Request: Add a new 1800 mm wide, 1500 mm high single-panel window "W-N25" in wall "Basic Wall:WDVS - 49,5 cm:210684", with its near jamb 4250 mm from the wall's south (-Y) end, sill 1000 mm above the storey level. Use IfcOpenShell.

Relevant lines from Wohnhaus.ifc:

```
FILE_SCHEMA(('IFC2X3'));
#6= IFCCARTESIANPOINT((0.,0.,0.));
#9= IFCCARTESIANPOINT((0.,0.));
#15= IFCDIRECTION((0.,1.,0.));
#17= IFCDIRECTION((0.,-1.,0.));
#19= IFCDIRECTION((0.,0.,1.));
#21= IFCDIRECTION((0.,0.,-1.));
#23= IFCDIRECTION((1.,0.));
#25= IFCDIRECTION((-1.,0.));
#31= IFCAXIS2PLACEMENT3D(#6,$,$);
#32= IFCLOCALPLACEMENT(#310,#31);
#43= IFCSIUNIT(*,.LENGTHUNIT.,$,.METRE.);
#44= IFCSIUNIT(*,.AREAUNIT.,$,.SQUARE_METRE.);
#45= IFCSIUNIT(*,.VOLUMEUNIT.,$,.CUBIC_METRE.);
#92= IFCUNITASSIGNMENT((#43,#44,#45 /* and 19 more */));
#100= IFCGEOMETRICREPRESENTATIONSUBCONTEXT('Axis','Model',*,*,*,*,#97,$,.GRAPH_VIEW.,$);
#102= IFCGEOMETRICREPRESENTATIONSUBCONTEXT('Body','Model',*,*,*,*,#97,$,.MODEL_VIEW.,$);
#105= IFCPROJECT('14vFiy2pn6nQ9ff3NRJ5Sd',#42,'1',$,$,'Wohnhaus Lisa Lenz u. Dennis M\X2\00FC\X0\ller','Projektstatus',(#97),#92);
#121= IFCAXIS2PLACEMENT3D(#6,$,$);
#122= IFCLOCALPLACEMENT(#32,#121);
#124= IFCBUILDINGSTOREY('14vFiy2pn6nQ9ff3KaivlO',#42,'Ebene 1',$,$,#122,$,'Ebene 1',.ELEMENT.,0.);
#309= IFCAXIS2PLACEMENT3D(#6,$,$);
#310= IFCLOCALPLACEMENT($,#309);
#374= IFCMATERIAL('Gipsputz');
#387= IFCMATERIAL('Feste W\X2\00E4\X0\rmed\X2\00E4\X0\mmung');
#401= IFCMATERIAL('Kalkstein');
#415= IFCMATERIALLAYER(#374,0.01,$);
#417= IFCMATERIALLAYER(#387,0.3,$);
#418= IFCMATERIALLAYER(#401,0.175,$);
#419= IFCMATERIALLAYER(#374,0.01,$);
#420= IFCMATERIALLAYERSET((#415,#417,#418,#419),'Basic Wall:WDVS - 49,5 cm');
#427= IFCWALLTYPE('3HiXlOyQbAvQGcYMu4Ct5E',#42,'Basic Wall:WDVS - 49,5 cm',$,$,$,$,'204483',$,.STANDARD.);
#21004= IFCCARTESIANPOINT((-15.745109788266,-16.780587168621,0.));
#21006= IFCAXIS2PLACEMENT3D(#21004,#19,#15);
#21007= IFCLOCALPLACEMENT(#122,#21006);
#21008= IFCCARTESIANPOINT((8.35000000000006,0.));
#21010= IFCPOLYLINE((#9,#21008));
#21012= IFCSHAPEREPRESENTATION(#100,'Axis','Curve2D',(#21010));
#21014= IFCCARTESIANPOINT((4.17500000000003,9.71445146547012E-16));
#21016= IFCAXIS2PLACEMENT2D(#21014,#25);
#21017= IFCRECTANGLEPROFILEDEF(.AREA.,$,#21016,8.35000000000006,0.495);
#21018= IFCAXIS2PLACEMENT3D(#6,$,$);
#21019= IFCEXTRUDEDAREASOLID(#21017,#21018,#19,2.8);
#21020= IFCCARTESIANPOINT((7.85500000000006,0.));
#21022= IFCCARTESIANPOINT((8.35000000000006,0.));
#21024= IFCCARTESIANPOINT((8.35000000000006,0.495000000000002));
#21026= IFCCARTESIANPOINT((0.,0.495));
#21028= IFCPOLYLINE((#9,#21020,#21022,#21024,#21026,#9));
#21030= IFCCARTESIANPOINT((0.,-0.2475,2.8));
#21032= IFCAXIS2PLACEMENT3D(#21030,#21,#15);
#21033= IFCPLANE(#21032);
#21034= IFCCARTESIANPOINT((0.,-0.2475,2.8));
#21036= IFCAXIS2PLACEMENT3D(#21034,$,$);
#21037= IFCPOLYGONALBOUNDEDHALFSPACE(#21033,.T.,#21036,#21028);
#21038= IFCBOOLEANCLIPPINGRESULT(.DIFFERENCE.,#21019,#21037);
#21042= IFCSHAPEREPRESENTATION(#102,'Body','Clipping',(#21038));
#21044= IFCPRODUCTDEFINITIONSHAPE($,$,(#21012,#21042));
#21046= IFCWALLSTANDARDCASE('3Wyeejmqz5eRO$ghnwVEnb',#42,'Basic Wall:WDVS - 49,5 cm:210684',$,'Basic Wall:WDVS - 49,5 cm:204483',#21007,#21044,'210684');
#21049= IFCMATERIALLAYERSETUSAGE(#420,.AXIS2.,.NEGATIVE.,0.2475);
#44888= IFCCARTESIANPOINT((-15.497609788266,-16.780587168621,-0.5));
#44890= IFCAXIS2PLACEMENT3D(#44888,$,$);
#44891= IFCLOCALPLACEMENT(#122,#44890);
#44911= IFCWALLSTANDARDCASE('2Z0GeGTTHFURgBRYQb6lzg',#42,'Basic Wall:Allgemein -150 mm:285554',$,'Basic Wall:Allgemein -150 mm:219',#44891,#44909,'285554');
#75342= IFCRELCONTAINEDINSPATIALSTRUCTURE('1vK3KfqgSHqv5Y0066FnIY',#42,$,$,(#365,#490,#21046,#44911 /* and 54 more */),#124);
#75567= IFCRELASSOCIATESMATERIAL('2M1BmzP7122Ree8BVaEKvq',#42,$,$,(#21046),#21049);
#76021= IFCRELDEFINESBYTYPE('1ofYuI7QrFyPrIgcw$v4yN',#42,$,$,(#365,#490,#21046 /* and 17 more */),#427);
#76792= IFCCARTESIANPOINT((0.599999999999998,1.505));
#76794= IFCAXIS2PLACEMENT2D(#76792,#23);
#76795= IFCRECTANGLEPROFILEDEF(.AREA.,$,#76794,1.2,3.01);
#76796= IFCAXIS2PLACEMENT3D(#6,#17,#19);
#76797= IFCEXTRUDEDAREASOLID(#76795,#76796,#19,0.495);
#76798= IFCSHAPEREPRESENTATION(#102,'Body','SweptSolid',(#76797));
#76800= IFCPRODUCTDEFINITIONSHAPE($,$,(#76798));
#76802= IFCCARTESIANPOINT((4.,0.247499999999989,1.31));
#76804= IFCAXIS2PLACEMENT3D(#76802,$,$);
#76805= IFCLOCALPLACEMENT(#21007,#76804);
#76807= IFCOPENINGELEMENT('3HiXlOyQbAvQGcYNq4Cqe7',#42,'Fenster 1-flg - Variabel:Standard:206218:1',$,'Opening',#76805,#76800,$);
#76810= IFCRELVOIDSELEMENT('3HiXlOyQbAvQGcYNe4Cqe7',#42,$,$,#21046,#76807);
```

```python
import numpy as np
import ifcopenshell
import ifcopenshell.api.feature
import ifcopenshell.api.geometry
import ifcopenshell.api.root
import ifcopenshell.api.spatial
import ifcopenshell.api.type
import ifcopenshell.geom
import ifcopenshell.util.element
import ifcopenshell.util.placement
import ifcopenshell.util.representation
import ifcopenshell.util.shape
import ifcopenshell.util.unit

model = ifcopenshell.open("Wohnhaus.ifc")
unit_scale = ifcopenshell.util.unit.calculate_unit_scale(model)
settings = ifcopenshell.geom.settings()


def volume(element):
    """Net volume in cubic metres, openings subtracted."""
    shape = ifcopenshell.geom.create_shape(settings, element)
    return ifcopenshell.util.shape.get_volume(shape.geometry)


wall = model.by_guid("3Wyeejmqz5eRO$ghnwVEnb")
storey = ifcopenshell.util.element.get_container(wall, ifc_class="IfcBuildingStorey")
context = ifcopenshell.util.representation.get_context(model, "Model", "Body", "MODEL_VIEW")
before = volume(wall)

width, height, from_end, sill = 1.8, 1.5, 4.25, 1  # metres

# The wall runs along its own X axis, and the end named is its -X end.
wall_shape = ifcopenshell.geom.create_shape(settings, wall)
x, y, z = ifcopenshell.util.shape.get_vertices(wall_shape.geometry).T
start = x.min() + from_end
face, thickness = float(y.min()), float(y.max() - y.min())
wall_matrix = ifcopenshell.util.placement.get_local_placement(wall.ObjectPlacement)
level = ifcopenshell.util.placement.get_local_placement(storey.ObjectPlacement)[2, 3]


def in_wall(x, y):
    """Placement at x, y metres in the wall's axes, at sill height."""
    matrix = wall_matrix.copy()
    matrix[:, 3] = wall_matrix @ np.array([x / unit_scale, y / unit_scale, 0.0, 1.0])
    matrix[2, 3] = level + sill / unit_scale
    return matrix


# Opening: a box that overshoots both wall faces by 50 mm.
opening = ifcopenshell.api.root.create_entity(model, ifc_class="IfcOpeningElement")
box = ifcopenshell.api.geometry.add_wall_representation(
    model, context=context, length=width, height=height, thickness=thickness + 0.1
)
ifcopenshell.api.geometry.assign_representation(model, product=opening, representation=box)
ifcopenshell.api.geometry.edit_object_placement(model, product=opening, matrix=in_wall(start, face - 0.05), is_si=False)
ifcopenshell.api.feature.add_feature(model, feature=opening, element=wall)

window = ifcopenshell.api.root.create_entity(model, ifc_class="IfcWindow", name="W-N25")
window.OverallWidth, window.OverallHeight = width / unit_scale, height / unit_scale
body = ifcopenshell.api.geometry.add_window_representation(
    model,
    context=context,
    overall_width=window.OverallWidth,
    overall_height=window.OverallHeight,
    partition_type="SINGLE_PANEL",
)
ifcopenshell.api.geometry.assign_representation(model, product=window, representation=body)
ifcopenshell.api.spatial.assign_container(model, products=[window], relating_structure=storey)
fills = ifcopenshell.api.feature.add_filling(model, opening=opening, element=window)
fills.OwnerHistory = window.OwnerHistory  # required in IFC2X3

# IFC2X3 keeps the operation on the window style.
style = ifcopenshell.api.root.create_entity(model, ifc_class="IfcWindowStyle", name="W-N25")
style.OperationType, style.ConstructionType = "SINGLE_PANEL", "NOTDEFINED"
style.ParameterTakesPrecedence = style.Sizeable = False
ifcopenshell.api.type.assign_type(model, related_objects=[window], relating_type=style)

# Centre the window in the wall's thickness.
ifcopenshell.api.geometry.edit_object_placement(model, product=window, matrix=in_wall(start, face), is_si=False)
window_shape = ifcopenshell.geom.create_shape(settings, window)
depth = ifcopenshell.util.shape.get_vertices(window_shape.geometry)[:, 1]
offset = face + thickness / 2 - (depth.min() + depth.max()) / 2
ifcopenshell.api.geometry.edit_object_placement(model, product=window, matrix=in_wall(start, offset), is_si=False)

after = volume(wall)

print(f"wall volume {before:.3f} -> {after:.3f} m3")

model.write("Wohnhaus_updated.ifc")
```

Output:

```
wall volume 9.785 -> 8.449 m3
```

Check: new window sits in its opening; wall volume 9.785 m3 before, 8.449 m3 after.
